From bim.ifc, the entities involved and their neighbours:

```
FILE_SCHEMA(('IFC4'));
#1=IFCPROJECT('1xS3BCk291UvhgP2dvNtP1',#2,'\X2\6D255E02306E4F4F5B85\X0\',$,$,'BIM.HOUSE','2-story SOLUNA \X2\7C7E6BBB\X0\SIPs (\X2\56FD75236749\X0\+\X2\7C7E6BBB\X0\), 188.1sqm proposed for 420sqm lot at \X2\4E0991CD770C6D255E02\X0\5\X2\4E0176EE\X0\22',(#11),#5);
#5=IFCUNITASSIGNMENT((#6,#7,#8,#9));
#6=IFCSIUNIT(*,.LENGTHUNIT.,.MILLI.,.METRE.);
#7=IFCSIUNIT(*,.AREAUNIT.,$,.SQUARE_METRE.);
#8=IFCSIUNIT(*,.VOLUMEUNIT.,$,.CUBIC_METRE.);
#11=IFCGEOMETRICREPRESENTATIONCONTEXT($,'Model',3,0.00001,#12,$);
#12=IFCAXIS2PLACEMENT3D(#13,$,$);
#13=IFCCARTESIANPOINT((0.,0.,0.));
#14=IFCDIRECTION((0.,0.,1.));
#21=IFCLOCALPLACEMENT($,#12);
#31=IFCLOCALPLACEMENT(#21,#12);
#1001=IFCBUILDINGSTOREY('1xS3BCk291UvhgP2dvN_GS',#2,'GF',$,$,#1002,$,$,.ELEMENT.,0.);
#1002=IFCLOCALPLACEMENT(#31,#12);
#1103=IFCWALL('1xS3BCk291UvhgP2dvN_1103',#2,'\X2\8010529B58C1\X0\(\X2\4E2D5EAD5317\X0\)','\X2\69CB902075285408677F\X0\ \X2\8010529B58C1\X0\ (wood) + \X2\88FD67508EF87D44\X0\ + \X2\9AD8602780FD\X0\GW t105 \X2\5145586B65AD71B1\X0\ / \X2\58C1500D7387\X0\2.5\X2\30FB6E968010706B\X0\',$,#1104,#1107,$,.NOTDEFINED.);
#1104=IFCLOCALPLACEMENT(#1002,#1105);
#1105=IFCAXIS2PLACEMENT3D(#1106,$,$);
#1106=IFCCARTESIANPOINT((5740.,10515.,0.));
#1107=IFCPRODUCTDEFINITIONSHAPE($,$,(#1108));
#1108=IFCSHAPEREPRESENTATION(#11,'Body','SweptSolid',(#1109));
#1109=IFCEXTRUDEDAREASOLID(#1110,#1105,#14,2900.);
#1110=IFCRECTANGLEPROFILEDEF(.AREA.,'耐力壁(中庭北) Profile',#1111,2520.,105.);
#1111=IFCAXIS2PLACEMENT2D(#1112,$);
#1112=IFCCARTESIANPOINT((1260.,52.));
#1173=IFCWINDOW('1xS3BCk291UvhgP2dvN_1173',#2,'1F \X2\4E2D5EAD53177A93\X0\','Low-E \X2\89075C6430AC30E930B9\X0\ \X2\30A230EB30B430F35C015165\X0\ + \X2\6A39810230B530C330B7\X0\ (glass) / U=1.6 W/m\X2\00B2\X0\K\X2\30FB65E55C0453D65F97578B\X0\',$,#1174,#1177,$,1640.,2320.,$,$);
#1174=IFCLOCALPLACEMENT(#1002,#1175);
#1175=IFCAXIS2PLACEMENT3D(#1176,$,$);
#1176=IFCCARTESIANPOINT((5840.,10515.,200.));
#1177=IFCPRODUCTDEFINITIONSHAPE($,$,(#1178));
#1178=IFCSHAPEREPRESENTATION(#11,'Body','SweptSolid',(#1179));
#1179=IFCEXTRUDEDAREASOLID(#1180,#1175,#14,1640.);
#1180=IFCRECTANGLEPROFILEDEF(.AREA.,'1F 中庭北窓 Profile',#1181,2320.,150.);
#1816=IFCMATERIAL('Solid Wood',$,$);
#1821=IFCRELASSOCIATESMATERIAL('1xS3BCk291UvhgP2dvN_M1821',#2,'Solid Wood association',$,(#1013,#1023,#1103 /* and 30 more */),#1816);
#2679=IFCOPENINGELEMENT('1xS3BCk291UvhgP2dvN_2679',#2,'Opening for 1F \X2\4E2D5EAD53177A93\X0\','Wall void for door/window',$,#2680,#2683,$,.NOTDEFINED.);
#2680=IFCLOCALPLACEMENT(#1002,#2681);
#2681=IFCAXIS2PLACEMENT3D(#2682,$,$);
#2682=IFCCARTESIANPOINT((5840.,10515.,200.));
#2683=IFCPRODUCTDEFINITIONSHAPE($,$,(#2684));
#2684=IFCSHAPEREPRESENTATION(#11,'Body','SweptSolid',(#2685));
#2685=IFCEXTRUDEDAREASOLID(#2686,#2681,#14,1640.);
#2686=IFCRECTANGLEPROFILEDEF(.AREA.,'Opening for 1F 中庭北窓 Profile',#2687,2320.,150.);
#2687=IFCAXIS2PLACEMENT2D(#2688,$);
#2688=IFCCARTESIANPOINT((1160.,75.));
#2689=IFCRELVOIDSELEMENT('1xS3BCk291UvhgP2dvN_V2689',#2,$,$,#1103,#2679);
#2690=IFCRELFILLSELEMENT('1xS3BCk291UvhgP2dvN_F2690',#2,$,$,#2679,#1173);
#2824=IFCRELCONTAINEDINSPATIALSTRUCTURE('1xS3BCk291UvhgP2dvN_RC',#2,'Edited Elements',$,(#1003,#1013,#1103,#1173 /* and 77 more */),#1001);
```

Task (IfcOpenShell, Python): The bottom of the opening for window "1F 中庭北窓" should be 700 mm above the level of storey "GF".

```python
import numpy as np
import ifcopenshell
import ifcopenshell.api.geometry
import ifcopenshell.geom
import ifcopenshell.util.element
import ifcopenshell.util.placement
import ifcopenshell.util.shape
import ifcopenshell.util.unit

model = ifcopenshell.open("bim.ifc")
unit_scale = ifcopenshell.util.unit.calculate_unit_scale(model)

window = model.by_guid("1xS3BCk291UvhgP2dvN_1173")
opening = window.FillsVoids[0].RelatingOpeningElement
storey = ifcopenshell.util.element.get_container(window, ifc_class="IfcBuildingStorey")
level = ifcopenshell.util.placement.get_local_placement(storey.ObjectPlacement)[2, 3]

# The opening's origin need not be at the sill, so measure its lowest point.
shape = ifcopenshell.geom.create_shape(ifcopenshell.geom.settings(), opening)
bottom = ifcopenshell.util.shape.get_shape_bottom_elevation(shape, shape.geometry) / unit_scale
dz = level + 700.0 - bottom

shift = np.array([0.0, 0.0, dz])
# The window is not placed relative to its opening, so move both.
for product in (opening, window):
    matrix = ifcopenshell.util.placement.get_local_placement(product.ObjectPlacement)
    matrix[:3, 3] += shift
    ifcopenshell.api.geometry.edit_object_placement(model, product=product, matrix=matrix, is_si=False)

print(f"moved by {dz * unit_scale:+.3f} m")

model.write("bim-out.ifc")
```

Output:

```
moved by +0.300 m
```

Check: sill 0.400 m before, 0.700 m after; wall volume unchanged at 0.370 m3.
